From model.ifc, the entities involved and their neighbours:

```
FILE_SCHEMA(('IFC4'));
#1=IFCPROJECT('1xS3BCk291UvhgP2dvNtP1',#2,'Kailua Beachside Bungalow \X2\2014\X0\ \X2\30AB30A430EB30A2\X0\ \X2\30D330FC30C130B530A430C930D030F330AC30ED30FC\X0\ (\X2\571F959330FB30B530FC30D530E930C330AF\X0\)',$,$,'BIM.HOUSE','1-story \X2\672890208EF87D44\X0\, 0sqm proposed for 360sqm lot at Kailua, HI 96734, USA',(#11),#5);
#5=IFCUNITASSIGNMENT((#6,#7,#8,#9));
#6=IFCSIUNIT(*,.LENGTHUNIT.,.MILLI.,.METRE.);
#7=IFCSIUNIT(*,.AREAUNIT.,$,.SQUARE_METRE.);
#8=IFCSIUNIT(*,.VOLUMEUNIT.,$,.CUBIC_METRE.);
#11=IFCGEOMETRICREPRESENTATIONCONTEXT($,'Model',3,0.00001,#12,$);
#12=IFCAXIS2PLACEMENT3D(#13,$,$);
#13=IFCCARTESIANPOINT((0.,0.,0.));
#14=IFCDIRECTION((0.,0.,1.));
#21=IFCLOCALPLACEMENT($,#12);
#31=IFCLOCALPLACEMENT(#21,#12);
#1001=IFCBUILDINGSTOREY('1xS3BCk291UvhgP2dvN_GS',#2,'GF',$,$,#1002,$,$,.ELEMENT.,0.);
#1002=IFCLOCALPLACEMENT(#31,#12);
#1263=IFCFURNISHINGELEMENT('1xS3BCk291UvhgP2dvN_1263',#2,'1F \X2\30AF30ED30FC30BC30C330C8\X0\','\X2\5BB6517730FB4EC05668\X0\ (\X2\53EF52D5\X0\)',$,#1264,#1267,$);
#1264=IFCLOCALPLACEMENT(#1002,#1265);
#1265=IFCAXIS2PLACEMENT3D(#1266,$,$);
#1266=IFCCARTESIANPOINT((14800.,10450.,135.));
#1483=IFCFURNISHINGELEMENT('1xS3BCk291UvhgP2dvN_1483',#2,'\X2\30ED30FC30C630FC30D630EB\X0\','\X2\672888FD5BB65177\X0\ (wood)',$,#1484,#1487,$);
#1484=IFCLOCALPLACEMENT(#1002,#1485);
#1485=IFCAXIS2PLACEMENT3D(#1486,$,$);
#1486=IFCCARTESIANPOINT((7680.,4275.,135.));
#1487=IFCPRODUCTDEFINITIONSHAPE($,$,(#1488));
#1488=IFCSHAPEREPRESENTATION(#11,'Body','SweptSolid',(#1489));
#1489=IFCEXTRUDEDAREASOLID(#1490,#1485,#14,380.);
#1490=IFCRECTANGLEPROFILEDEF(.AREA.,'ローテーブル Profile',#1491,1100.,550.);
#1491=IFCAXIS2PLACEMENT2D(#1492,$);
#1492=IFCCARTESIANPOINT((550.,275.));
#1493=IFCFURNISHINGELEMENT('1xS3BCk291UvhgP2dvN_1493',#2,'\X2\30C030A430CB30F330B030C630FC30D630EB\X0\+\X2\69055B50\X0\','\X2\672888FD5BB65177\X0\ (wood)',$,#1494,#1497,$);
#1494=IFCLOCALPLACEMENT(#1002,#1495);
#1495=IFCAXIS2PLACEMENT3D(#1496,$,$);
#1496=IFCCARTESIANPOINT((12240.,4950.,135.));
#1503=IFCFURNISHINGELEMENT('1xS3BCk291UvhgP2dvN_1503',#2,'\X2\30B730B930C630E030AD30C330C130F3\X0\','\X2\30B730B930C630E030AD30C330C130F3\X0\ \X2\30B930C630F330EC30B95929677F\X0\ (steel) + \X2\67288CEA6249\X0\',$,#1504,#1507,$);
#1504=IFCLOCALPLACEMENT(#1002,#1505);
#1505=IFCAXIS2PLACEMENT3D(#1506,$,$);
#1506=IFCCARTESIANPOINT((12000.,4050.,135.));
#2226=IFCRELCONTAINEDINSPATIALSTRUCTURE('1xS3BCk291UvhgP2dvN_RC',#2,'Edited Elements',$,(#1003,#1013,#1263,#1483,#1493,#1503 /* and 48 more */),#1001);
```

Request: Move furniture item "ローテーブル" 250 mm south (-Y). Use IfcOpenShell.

```python
import ifcopenshell
import ifcopenshell.api.geometry
import ifcopenshell.util.placement

model = ifcopenshell.open("model.ifc")

item = model.by_id(1483)
matrix = ifcopenshell.util.placement.get_local_placement(item.ObjectPlacement)
matrix[1, 3] -= 250.0
ifcopenshell.api.geometry.edit_object_placement(model, product=item, matrix=matrix, is_si=False)

print(ifcopenshell.util.placement.get_local_placement(item.ObjectPlacement).round(3) + 0.0)

model.write("model_updated.ifc")
```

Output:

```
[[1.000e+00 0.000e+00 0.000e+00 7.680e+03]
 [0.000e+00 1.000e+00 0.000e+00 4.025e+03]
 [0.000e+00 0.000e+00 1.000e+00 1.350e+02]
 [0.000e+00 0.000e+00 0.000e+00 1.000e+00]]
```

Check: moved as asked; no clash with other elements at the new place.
